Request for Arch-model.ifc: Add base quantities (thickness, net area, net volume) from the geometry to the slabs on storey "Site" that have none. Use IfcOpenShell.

First a look at what the model holds.

```python
import ifcopenshell
import ifcopenshell.util.element
import ifcopenshell.util.unit

model = ifcopenshell.open("Arch-model.ifc")
print(model.schema)
for unit_type in ("LENGTHUNIT", "AREAUNIT", "VOLUMEUNIT"):
    print(unit_type, ifcopenshell.util.unit.calculate_unit_scale(model, unit_type))
storey = next(s for s in model.by_type("IfcBuildingStorey") if s.Name == "Site")
slabs = [e for e in ifcopenshell.util.element.get_decomposition(storey) if e.is_a("IfcSlab")]
for e in sorted(slabs, key=lambda e: e.id()):
    print(e.id(), e.is_a(), e.Name, list(ifcopenshell.util.element.get_psets(e, qtos_only=True)), sep=" | ")
```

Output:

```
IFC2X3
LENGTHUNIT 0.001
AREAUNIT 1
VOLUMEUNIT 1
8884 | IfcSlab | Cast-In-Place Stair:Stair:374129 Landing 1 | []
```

```python
import ifcopenshell
import ifcopenshell.api.pset
import ifcopenshell.geom
import ifcopenshell.util.element
import ifcopenshell.util.shape
import ifcopenshell.util.unit

model = ifcopenshell.open("Arch-model.ifc")
unit_scale = ifcopenshell.util.unit.calculate_unit_scale(model)
area_scale = ifcopenshell.util.unit.calculate_unit_scale(model, "AREAUNIT")
volume_scale = ifcopenshell.util.unit.calculate_unit_scale(model, "VOLUMEUNIT")
settings = ifcopenshell.geom.settings()

storey = next(s for s in model.by_type("IfcBuildingStorey") if s.Name == "Site")
slabs = [e for e in ifcopenshell.util.element.get_decomposition(storey) if e.is_a("IfcSlab")]

for e in sorted(slabs, key=lambda e: e.id()):
    if ifcopenshell.util.element.get_psets(e, qtos_only=True, should_inherit=False):
        continue
    # Geometry comes back in metres, in the element's own axes.
    shape = ifcopenshell.geom.create_shape(settings, e)
    values = {
        "Width": ifcopenshell.util.shape.get_z(shape.geometry) / unit_scale,
        "NetArea": ifcopenshell.util.shape.get_footprint_area(shape.geometry) / area_scale,
        "NetVolume": ifcopenshell.util.shape.get_volume(shape.geometry) / volume_scale,
    }
    qto = ifcopenshell.api.pset.add_qto(model, product=e, name="BaseQuantities")
    ifcopenshell.api.pset.edit_qto(model, qto=qto, properties=values)
    print(e.id(), {k: round(v, 3) for k, v in values.items()})

model.write("Arch-model_updated.ifc")
```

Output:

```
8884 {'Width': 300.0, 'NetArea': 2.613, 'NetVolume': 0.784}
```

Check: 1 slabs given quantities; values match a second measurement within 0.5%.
